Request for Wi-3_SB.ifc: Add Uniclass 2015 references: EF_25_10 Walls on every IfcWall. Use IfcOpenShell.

First a look at what the model holds.

```python
import ifcopenshell

model = ifcopenshell.open("Wi-3_SB.ifc")
print(model.schema)
print("classifications:", [c.Name for c in model.by_type("IfcClassification")])
for ifc_class in ("IfcDoor", "IfcRoof", "IfcStair", "IfcWall", "IfcWindow"):
    print(ifc_class, len(model.by_type(ifc_class)))
```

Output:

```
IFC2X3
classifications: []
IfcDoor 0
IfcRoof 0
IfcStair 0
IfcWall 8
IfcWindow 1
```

```python
import ifcopenshell
import ifcopenshell.api.classification

model = ifcopenshell.open("Wi-3_SB.ifc")

# IFC2X3 requires Source and Edition and has no link from the project to the system.
system = model.create_entity("IfcClassification", Source="NBS", Edition="2015", Name="Uniclass 2015")

codes = {
    "IfcWall": ("EF_25_10", "Walls"),
}
for ifc_class, (code, name) in codes.items():
    products = model.by_type(ifc_class)
    ifcopenshell.api.classification.add_reference(
        model, products=products, classification=system, identification=code, name=name
    )
    print(code, len(products))

model.write("Wi-3_SB_updated.ifc")
```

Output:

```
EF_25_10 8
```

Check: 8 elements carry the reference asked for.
